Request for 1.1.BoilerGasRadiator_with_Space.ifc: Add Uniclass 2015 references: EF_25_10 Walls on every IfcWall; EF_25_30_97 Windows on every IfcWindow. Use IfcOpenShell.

First a look at what the model holds.

```python
import ifcopenshell

model = ifcopenshell.open("1.1.BoilerGasRadiator_with_Space.ifc")
print(model.schema)
print("classifications:", [c.Name for c in model.by_type("IfcClassification")])
for ifc_class in ("IfcDoor", "IfcRoof", "IfcStair", "IfcWall", "IfcWindow"):
    print(ifc_class, len(model.by_type(ifc_class)))
```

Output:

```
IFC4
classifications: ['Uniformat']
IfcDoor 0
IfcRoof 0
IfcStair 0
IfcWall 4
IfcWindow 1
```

```python
import ifcopenshell
import ifcopenshell.api.classification

model = ifcopenshell.open("1.1.BoilerGasRadiator_with_Space.ifc")

system = ifcopenshell.api.classification.add_classification(model, classification="Uniclass 2015")

codes = {
    "IfcWall": ("EF_25_10", "Walls"),
    "IfcWindow": ("EF_25_30_97", "Windows"),
}
for ifc_class, (code, name) in codes.items():
    products = model.by_type(ifc_class)
    ifcopenshell.api.classification.add_reference(
        model, products=products, classification=system, identification=code, name=name
    )
    print(code, len(products))

model.write("1.1.BoilerGasRadiator_with_Space-out.ifc")
```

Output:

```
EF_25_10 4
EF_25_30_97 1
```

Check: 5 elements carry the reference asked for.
